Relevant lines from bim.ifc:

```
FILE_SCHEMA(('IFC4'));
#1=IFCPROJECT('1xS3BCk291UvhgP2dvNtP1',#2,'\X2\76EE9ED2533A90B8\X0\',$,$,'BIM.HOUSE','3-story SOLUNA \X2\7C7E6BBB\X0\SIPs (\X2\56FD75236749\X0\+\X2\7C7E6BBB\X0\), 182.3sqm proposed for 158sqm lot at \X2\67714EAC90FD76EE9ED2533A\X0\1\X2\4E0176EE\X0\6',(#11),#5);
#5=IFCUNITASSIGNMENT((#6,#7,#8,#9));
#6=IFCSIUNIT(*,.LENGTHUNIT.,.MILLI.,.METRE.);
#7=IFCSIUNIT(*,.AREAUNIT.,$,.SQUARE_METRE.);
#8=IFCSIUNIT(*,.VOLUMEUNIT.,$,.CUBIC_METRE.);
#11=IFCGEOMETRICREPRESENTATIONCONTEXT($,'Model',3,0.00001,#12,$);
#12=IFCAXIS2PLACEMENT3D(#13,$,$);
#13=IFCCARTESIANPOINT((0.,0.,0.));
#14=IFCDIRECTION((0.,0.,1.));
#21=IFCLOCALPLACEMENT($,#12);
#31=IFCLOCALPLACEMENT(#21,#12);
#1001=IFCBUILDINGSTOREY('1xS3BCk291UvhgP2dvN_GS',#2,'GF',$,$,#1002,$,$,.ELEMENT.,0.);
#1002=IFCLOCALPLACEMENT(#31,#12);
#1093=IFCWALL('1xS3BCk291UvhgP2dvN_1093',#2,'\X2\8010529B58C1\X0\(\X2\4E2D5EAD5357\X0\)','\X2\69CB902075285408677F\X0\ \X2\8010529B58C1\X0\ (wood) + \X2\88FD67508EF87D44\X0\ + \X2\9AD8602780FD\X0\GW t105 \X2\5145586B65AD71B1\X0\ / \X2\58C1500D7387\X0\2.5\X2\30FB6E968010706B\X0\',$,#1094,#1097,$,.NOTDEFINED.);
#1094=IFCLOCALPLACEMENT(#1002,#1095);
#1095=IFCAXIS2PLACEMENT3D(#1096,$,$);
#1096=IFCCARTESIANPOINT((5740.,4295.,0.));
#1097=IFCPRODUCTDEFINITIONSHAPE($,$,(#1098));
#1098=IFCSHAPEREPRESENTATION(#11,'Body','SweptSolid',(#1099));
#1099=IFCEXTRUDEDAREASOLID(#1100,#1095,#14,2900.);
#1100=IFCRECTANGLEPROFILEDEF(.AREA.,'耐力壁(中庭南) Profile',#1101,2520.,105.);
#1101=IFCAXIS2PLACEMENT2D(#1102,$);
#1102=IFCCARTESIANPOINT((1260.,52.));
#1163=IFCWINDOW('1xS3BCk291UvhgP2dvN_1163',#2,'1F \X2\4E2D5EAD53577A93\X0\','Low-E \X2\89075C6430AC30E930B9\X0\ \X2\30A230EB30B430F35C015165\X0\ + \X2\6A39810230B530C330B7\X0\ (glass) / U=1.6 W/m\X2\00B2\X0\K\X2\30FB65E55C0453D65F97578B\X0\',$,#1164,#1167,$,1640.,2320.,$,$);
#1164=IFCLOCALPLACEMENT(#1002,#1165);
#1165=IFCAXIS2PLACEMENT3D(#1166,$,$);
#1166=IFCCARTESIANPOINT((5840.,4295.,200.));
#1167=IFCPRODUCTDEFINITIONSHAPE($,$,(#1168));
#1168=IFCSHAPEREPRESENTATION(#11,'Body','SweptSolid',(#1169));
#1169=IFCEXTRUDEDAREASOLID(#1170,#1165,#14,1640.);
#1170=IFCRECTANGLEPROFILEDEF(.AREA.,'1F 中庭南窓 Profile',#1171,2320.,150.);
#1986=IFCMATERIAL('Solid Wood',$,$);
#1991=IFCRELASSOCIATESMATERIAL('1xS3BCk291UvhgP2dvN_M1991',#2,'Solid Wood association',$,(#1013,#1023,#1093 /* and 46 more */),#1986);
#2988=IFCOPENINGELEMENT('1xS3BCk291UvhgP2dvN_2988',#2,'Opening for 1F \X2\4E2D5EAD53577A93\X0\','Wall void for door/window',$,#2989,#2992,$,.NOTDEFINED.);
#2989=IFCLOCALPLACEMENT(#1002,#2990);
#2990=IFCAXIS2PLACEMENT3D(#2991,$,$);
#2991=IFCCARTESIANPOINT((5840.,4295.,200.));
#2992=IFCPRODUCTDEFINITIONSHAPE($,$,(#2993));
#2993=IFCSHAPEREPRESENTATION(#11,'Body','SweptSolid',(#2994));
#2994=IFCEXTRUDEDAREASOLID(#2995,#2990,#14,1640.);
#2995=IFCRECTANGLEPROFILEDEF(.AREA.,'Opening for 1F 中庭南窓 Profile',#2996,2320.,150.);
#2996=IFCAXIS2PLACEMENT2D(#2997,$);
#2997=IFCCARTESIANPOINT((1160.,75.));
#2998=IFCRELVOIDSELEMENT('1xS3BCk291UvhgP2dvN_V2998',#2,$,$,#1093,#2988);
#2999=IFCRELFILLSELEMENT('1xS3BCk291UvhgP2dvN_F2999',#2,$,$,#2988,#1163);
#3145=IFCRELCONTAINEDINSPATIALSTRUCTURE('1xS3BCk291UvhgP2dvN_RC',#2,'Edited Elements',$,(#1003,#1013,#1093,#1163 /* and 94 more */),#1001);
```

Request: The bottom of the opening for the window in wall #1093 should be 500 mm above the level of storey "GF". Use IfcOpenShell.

```python
import numpy as np
import ifcopenshell
import ifcopenshell.api.geometry
import ifcopenshell.geom
import ifcopenshell.util.element
import ifcopenshell.util.placement
import ifcopenshell.util.shape
import ifcopenshell.util.unit

model = ifcopenshell.open("bim.ifc")
unit_scale = ifcopenshell.util.unit.calculate_unit_scale(model)

window = model.by_guid("1xS3BCk291UvhgP2dvN_1163")
opening = window.FillsVoids[0].RelatingOpeningElement
storey = ifcopenshell.util.element.get_container(window, ifc_class="IfcBuildingStorey")
level = ifcopenshell.util.placement.get_local_placement(storey.ObjectPlacement)[2, 3]

# The opening's origin need not be at the sill, so measure its lowest point.
shape = ifcopenshell.geom.create_shape(ifcopenshell.geom.settings(), opening)
bottom = ifcopenshell.util.shape.get_shape_bottom_elevation(shape, shape.geometry) / unit_scale
dz = level + 0.5 / unit_scale - bottom

shift = np.array([0.0, 0.0, dz])
# The window is not placed relative to its opening, so move both.
for product in (opening, window):
    matrix = ifcopenshell.util.placement.get_local_placement(product.ObjectPlacement)
    matrix[:3, 3] += shift
    ifcopenshell.api.geometry.edit_object_placement(model, product=product, matrix=matrix, is_si=False)

print(f"moved by {dz * unit_scale:+.3f} m")

model.write("bim-out.ifc")
```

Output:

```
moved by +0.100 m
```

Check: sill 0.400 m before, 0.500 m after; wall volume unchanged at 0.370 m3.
